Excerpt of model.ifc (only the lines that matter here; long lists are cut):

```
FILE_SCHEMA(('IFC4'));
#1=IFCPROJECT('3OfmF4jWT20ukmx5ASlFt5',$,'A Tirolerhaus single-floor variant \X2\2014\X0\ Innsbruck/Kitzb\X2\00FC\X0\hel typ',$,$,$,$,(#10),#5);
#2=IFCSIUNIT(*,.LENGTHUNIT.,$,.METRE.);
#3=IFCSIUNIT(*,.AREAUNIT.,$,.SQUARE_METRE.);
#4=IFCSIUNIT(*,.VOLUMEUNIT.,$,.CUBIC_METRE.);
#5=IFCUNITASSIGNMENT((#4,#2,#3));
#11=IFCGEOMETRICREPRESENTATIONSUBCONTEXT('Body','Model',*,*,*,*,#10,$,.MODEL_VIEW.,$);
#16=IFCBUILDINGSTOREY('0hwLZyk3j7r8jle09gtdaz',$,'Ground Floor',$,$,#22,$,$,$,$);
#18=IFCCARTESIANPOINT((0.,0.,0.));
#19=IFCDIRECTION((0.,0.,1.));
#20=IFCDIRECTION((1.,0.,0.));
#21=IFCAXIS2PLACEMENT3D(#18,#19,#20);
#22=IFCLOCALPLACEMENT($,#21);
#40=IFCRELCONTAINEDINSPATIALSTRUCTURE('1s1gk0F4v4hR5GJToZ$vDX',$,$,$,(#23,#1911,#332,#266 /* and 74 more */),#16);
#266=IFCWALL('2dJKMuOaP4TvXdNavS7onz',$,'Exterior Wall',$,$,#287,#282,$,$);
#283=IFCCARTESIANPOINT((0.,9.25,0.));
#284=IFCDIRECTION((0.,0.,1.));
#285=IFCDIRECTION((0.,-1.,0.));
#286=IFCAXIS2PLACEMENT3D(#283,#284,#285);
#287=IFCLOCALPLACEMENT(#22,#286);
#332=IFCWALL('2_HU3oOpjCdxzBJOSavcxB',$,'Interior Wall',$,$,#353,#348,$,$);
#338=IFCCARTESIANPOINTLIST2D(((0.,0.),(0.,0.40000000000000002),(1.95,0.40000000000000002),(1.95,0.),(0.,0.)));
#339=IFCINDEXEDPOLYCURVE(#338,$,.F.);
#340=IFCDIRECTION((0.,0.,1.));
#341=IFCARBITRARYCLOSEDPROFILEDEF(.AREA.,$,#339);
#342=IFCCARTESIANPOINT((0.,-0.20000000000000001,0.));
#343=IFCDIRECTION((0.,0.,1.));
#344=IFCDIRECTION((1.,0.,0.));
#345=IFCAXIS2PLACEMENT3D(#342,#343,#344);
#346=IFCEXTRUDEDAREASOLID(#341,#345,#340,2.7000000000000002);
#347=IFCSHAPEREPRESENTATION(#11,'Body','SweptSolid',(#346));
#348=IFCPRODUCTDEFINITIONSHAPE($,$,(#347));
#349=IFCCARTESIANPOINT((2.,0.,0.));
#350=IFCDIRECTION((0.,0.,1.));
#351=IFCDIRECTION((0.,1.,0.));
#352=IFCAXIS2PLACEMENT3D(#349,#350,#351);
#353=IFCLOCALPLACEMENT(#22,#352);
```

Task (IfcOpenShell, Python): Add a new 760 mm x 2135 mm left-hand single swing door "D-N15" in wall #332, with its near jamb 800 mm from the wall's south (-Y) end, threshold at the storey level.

```python
import numpy as np
import ifcopenshell
import ifcopenshell.api.feature
import ifcopenshell.api.geometry
import ifcopenshell.api.root
import ifcopenshell.api.spatial
import ifcopenshell.geom
import ifcopenshell.util.element
import ifcopenshell.util.placement
import ifcopenshell.util.representation
import ifcopenshell.util.shape
import ifcopenshell.util.unit

model = ifcopenshell.open("model.ifc")
unit_scale = ifcopenshell.util.unit.calculate_unit_scale(model)
settings = ifcopenshell.geom.settings()


def volume(element):
    """Net volume in cubic metres, openings subtracted."""
    shape = ifcopenshell.geom.create_shape(settings, element)
    return ifcopenshell.util.shape.get_volume(shape.geometry)


wall = model.by_guid("2_HU3oOpjCdxzBJOSavcxB")
storey = ifcopenshell.util.element.get_container(wall, ifc_class="IfcBuildingStorey")
context = ifcopenshell.util.representation.get_context(model, "Model", "Body", "MODEL_VIEW")
before = volume(wall)

width, height, from_end, sill = 0.76, 2.135, 0.8, 0.0  # metres

# The wall runs along its own X axis, and the end named is its -X end.
wall_shape = ifcopenshell.geom.create_shape(settings, wall)
x, y, z = ifcopenshell.util.shape.get_vertices(wall_shape.geometry).T
start = x.min() + from_end
face, thickness = float(y.min()), float(y.max() - y.min())
wall_matrix = ifcopenshell.util.placement.get_local_placement(wall.ObjectPlacement)
level = ifcopenshell.util.placement.get_local_placement(storey.ObjectPlacement)[2, 3]


def in_wall(x, y):
    """Placement at x, y metres in the wall's axes, at sill height."""
    matrix = wall_matrix.copy()
    matrix[:, 3] = wall_matrix @ np.array([x / unit_scale, y / unit_scale, 0.0, 1.0])
    matrix[2, 3] = level + sill / unit_scale
    return matrix


# Opening: a box that overshoots both wall faces by 50 mm.
opening = ifcopenshell.api.root.create_entity(model, ifc_class="IfcOpeningElement", predefined_type="OPENING")
box = ifcopenshell.api.geometry.add_wall_representation(
    model, context=context, length=width, height=height, thickness=thickness + 0.1
)
ifcopenshell.api.geometry.assign_representation(model, product=opening, representation=box)
ifcopenshell.api.geometry.edit_object_placement(model, product=opening, matrix=in_wall(start, face - 0.05), is_si=False)
ifcopenshell.api.feature.add_feature(model, feature=opening, element=wall)

door = ifcopenshell.api.root.create_entity(model, ifc_class="IfcDoor", name="D-N15", predefined_type="DOOR")
door.OverallWidth, door.OverallHeight = width / unit_scale, height / unit_scale
door.OperationType = "SINGLE_SWING_LEFT"
body = ifcopenshell.api.geometry.add_door_representation(
    model,
    context=context,
    overall_width=door.OverallWidth,
    overall_height=door.OverallHeight,
    operation_type="SINGLE_SWING_LEFT",
    lining_properties={"LiningDepth": thickness / unit_scale, "ThresholdDepth": thickness / unit_scale},
)
ifcopenshell.api.geometry.assign_representation(model, product=door, representation=body)
ifcopenshell.api.spatial.assign_container(model, products=[door], relating_structure=storey)
ifcopenshell.api.feature.add_filling(model, opening=opening, element=door)

# The lining spans the wall, so the door starts at the wall face.
ifcopenshell.api.geometry.edit_object_placement(model, product=door, matrix=in_wall(start, face), is_si=False)

after = volume(wall)

print(f"wall volume {before:.3f} -> {after:.3f} m3")

model.write("model_v2.ifc")
```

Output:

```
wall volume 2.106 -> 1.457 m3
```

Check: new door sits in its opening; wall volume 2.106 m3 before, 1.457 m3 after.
